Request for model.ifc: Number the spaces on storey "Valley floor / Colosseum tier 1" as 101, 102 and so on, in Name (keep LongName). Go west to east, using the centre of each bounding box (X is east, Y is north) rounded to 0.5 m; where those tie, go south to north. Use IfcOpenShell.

First a look at what the model holds.

```python
import ifcopenshell
import ifcopenshell.util.element
import ifcopenshell.util.placement

model = ifcopenshell.open("model.ifc")
print(model.schema)
storey = next(s for s in model.by_type("IfcBuildingStorey") if s.Name == "Valley floor / Colosseum tier 1")
spaces = [e for e in ifcopenshell.util.element.get_decomposition(storey) if e.is_a("IfcSpace")]
for e in sorted(spaces, key=lambda e: e.id()):
    origin = ifcopenshell.util.placement.get_local_placement(e.ObjectPlacement)[:3, 3]
    print(e.id(), e.Name, e.LongName, origin.round(2) + 0.0, sep=" | ")
```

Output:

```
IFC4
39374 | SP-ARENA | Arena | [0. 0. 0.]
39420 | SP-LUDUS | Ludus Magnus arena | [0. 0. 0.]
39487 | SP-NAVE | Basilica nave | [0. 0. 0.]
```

```python
import ifcopenshell
import ifcopenshell.geom
import ifcopenshell.util.element
import ifcopenshell.util.shape

model = ifcopenshell.open("model.ifc")
settings = ifcopenshell.geom.settings()
settings.set("use-world-coords", True)


def centre(element):
    shape = ifcopenshell.geom.create_shape(settings, element)
    return ifcopenshell.util.shape.get_bbox_centroid(shape.geometry)


storey = next(s for s in model.by_type("IfcBuildingStorey") if s.Name == "Valley floor / Colosseum tier 1")
spaces = [e for e in ifcopenshell.util.element.get_decomposition(storey) if e.is_a("IfcSpace")]

# Insertion points can sit at a corner or the storey origin, so sort by the geometry (in metres).
centres = {e: centre(e) for e in spaces}
spaces.sort(key=lambda e: (round(centres[e][0] / 0.5), centres[e][1]))

for i, e in enumerate(spaces, start=1):
    number = f"1{i:02d}"
    e.Name = number
    print(e.id(), number)

model.write("model_v2.ifc")
```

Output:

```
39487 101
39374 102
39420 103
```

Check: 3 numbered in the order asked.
